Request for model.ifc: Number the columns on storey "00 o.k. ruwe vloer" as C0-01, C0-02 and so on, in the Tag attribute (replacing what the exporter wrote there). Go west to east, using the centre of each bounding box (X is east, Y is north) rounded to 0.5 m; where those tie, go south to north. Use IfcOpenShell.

First a look at what the model holds.

```python
import ifcopenshell
import ifcopenshell.util.element
import ifcopenshell.util.placement

model = ifcopenshell.open("model.ifc")
print(model.schema)
storey = next(s for s in model.by_type("IfcBuildingStorey") if s.Name == "00 o.k. ruwe vloer")
columns = [e for e in ifcopenshell.util.element.get_decomposition(storey) if e.is_a("IfcColumn")]
for e in sorted(columns, key=lambda e: e.id()):
    origin = ifcopenshell.util.placement.get_local_placement(e.ObjectPlacement)[:3, 3]
    print(e.id(), e.Tag, e.Name, origin.round(2) + 0.0, sep=" | ")
```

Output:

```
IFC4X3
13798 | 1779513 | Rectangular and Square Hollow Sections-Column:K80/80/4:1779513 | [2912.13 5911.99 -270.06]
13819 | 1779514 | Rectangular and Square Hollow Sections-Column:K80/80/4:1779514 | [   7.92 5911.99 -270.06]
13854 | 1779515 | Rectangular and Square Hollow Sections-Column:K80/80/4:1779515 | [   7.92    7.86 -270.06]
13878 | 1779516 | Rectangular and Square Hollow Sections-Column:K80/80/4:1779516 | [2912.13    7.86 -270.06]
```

```python
import ifcopenshell
import ifcopenshell.geom
import ifcopenshell.util.element
import ifcopenshell.util.shape

model = ifcopenshell.open("model.ifc")
settings = ifcopenshell.geom.settings()
settings.set("use-world-coords", True)


def centre(element):
    shape = ifcopenshell.geom.create_shape(settings, element)
    return ifcopenshell.util.shape.get_bbox_centroid(shape.geometry)


storey = next(s for s in model.by_type("IfcBuildingStorey") if s.Name == "00 o.k. ruwe vloer")
columns = [e for e in ifcopenshell.util.element.get_decomposition(storey) if e.is_a("IfcColumn")]

# Insertion points can sit at a corner or the storey origin, so sort by the geometry (in metres).
centres = {e: centre(e) for e in columns}
columns.sort(key=lambda e: (round(centres[e][0] / 0.5), centres[e][1]))

for i, e in enumerate(columns, start=1):
    number = f"C0-{i:02d}"
    e.Tag = number
    print(e.id(), number)

model.write("model_rev.ifc")
```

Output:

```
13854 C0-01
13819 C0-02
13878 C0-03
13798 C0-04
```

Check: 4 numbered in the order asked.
